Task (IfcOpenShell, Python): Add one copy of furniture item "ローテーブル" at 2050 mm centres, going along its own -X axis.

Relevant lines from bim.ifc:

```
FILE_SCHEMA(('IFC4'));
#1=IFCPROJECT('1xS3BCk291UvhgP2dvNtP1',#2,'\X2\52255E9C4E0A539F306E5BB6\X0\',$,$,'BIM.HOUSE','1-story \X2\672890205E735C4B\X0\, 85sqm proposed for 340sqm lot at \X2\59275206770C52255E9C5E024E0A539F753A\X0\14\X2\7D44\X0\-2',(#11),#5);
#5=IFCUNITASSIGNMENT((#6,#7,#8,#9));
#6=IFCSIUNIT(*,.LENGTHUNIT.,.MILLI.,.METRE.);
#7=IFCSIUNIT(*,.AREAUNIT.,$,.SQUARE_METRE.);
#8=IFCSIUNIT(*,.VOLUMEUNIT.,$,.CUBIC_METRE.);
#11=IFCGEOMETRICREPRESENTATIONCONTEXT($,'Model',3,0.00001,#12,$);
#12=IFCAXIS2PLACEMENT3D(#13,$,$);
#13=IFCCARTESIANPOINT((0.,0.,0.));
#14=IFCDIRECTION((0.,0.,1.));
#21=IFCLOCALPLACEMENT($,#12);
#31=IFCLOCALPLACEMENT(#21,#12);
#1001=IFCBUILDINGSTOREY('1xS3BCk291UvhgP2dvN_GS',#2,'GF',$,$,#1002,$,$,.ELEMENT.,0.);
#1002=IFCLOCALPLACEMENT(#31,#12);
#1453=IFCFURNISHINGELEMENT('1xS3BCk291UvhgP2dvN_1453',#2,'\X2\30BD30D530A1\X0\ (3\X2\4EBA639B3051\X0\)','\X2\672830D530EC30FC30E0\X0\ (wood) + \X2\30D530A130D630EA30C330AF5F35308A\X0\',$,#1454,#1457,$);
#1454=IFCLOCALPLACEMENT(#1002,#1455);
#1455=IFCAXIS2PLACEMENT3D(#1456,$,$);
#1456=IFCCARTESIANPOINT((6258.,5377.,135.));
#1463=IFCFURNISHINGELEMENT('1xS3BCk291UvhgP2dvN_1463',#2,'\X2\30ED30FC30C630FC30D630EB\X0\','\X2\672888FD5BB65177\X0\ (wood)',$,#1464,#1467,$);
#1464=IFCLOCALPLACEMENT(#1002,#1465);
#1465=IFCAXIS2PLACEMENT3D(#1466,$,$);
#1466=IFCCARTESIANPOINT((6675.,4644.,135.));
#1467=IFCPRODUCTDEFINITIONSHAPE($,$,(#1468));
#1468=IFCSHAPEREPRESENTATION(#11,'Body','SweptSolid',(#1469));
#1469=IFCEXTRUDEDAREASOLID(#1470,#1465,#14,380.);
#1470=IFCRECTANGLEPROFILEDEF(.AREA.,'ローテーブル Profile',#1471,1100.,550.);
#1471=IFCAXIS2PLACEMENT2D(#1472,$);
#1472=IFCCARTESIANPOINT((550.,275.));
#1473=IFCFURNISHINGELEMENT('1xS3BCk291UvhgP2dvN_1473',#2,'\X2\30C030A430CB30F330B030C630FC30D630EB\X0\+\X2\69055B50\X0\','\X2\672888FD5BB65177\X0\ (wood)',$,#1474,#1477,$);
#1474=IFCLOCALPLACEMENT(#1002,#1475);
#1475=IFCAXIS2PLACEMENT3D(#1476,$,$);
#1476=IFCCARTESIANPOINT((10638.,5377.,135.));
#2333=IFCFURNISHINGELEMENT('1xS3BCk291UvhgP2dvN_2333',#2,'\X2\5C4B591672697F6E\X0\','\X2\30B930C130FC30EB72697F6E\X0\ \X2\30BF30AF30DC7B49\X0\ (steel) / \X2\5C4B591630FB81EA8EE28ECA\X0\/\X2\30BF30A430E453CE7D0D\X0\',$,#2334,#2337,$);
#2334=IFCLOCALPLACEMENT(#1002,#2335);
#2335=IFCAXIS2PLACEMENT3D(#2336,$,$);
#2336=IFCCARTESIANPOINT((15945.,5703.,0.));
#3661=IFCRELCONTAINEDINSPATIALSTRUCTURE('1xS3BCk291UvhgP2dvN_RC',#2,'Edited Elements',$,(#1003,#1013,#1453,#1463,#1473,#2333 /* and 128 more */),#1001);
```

```python
import ifcopenshell
import ifcopenshell.api.geometry
import ifcopenshell.api.root
import ifcopenshell.util.element
import ifcopenshell.util.placement
import ifcopenshell.util.unit

model = ifcopenshell.open("bim.ifc")
unit_scale = ifcopenshell.util.unit.calculate_unit_scale(model)


def reuse_history(source, copy):
    """copy_class also copies each property set's owner history, people and application; keep the originals."""
    for rel in copy.IsDefinedBy:
        if rel.is_a("IfcRelDefinesByProperties") and (history := rel.RelatingPropertyDefinition.OwnerHistory):
            rel.RelatingPropertyDefinition.OwnerHistory = source.OwnerHistory
            ifcopenshell.util.element.remove_deep2(model, history)


source = model.by_id(1463)
base = ifcopenshell.util.placement.get_local_placement(source.ObjectPlacement)
step = -base[:3, 0] * 2.05 / unit_scale

for i in range(1, 2):
    copy = ifcopenshell.api.root.copy_class(model, product=source)
    copy.Representation = ifcopenshell.util.element.copy_deep(
        model, source.Representation, exclude=["IfcGeometricRepresentationContext", "IfcRepresentationMap"]
    )
    reuse_history(source, copy)
    matrix = base.copy()
    matrix[:3, 3] += i * step
    print("added at", matrix[:3, 3].round(3) + 0.0)
    ifcopenshell.api.geometry.edit_object_placement(model, product=copy, matrix=matrix, is_si=False)

model.write("bim-out.ifc")
```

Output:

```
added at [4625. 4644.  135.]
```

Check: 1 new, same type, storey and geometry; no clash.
